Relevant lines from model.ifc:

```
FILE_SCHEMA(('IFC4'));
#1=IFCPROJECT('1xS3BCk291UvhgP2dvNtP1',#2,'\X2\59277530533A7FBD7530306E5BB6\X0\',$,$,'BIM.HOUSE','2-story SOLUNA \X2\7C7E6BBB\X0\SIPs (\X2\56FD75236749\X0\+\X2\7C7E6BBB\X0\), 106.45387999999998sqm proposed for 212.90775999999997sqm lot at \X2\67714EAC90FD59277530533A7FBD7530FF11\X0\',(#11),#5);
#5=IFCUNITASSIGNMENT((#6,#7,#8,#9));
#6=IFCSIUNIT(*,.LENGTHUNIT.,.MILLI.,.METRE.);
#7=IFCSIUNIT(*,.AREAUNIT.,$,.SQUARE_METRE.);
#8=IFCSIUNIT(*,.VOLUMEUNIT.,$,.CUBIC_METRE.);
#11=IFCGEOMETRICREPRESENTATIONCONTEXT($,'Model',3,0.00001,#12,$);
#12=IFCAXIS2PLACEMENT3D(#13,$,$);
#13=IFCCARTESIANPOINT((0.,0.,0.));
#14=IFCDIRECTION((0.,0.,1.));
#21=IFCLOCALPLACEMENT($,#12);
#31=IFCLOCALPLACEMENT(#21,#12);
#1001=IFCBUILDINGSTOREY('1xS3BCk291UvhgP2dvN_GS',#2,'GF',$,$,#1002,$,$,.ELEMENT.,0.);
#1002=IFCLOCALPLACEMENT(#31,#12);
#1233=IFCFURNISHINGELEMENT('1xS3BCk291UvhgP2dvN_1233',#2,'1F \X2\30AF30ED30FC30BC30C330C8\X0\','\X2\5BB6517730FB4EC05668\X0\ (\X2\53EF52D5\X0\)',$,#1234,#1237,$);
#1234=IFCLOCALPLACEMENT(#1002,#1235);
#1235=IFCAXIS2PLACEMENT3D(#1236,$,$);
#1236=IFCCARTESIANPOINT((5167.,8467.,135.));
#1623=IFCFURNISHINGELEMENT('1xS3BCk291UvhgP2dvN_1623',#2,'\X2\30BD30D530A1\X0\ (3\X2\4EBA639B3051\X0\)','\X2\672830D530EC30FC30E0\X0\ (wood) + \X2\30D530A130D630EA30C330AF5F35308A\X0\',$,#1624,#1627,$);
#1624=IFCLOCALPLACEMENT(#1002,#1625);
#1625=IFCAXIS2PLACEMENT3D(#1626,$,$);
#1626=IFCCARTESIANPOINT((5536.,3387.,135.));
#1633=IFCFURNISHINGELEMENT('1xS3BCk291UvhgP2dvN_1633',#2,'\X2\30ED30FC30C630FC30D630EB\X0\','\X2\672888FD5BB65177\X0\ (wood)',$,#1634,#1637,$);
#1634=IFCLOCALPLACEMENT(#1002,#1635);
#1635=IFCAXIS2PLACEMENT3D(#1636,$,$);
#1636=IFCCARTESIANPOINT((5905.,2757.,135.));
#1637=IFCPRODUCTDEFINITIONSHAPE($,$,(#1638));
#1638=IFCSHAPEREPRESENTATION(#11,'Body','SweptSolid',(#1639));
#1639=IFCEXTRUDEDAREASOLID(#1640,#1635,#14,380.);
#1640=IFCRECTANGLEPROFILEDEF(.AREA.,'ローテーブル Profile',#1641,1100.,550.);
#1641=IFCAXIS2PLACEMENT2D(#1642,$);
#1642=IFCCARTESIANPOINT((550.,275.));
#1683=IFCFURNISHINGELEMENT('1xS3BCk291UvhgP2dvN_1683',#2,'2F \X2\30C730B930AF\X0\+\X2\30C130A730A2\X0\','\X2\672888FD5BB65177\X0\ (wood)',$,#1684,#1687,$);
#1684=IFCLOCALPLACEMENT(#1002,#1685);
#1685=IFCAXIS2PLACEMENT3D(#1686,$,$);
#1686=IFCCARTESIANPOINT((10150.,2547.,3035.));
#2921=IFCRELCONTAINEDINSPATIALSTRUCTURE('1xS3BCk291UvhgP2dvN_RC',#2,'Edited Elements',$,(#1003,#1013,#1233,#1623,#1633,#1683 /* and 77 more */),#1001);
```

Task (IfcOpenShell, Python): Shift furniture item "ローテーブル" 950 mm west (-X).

```python
import ifcopenshell
import ifcopenshell.api.geometry
import ifcopenshell.util.placement
import ifcopenshell.util.unit

model = ifcopenshell.open("model.ifc")
unit_scale = ifcopenshell.util.unit.calculate_unit_scale(model)

item = model.by_guid("1xS3BCk291UvhgP2dvN_1633")
matrix = ifcopenshell.util.placement.get_local_placement(item.ObjectPlacement)
matrix[0, 3] -= 0.95 / unit_scale
ifcopenshell.api.geometry.edit_object_placement(model, product=item, matrix=matrix, is_si=False)

print(ifcopenshell.util.placement.get_local_placement(item.ObjectPlacement).round(3) + 0.0)

model.write("model_v2.ifc")
```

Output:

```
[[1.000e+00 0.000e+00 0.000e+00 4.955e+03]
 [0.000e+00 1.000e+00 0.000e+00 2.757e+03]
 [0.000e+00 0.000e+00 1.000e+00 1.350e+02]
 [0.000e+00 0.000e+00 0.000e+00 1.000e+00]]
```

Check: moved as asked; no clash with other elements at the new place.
